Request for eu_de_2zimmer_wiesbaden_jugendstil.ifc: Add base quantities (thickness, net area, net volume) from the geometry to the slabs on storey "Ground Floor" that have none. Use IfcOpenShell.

First a look at what the model holds.

```python
import ifcopenshell
import ifcopenshell.util.element
import ifcopenshell.util.unit

model = ifcopenshell.open("eu_de_2zimmer_wiesbaden_jugendstil.ifc")
print(model.schema)
for unit_type in ("LENGTHUNIT", "AREAUNIT", "VOLUMEUNIT"):
    print(unit_type, ifcopenshell.util.unit.calculate_unit_scale(model, unit_type))
storey = next(s for s in model.by_type("IfcBuildingStorey") if s.Name == "Ground Floor")
slabs = [e for e in ifcopenshell.util.element.get_decomposition(storey) if e.is_a("IfcSlab")]
for e in sorted(slabs, key=lambda e: e.id()):
    print(e.id(), e.is_a(), e.Name, list(ifcopenshell.util.element.get_psets(e, qtos_only=True)), sep=" | ")
```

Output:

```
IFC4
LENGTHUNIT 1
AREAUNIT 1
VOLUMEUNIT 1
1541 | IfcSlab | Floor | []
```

```python
import ifcopenshell
import ifcopenshell.api.pset
import ifcopenshell.geom
import ifcopenshell.util.element
import ifcopenshell.util.shape
import ifcopenshell.util.unit

model = ifcopenshell.open("eu_de_2zimmer_wiesbaden_jugendstil.ifc")
unit_scale = ifcopenshell.util.unit.calculate_unit_scale(model)
area_scale = ifcopenshell.util.unit.calculate_unit_scale(model, "AREAUNIT")
volume_scale = ifcopenshell.util.unit.calculate_unit_scale(model, "VOLUMEUNIT")
settings = ifcopenshell.geom.settings()

storey = next(s for s in model.by_type("IfcBuildingStorey") if s.Name == "Ground Floor")
slabs = [e for e in ifcopenshell.util.element.get_decomposition(storey) if e.is_a("IfcSlab")]

for e in sorted(slabs, key=lambda e: e.id()):
    if ifcopenshell.util.element.get_psets(e, qtos_only=True, should_inherit=False):
        continue
    # Geometry comes back in metres, in the element's own axes.
    shape = ifcopenshell.geom.create_shape(settings, e)
    values = {
        "Width": ifcopenshell.util.shape.get_z(shape.geometry) / unit_scale,
        "NetArea": ifcopenshell.util.shape.get_footprint_area(shape.geometry) / area_scale,
        "NetVolume": ifcopenshell.util.shape.get_volume(shape.geometry) / volume_scale,
    }
    qto = ifcopenshell.api.pset.add_qto(model, product=e, name="Qto_SlabBaseQuantities")
    ifcopenshell.api.pset.edit_qto(model, qto=qto, properties=values)
    print(e.id(), {k: round(v, 3) for k, v in values.items()})

model.write("eu_de_2zimmer_wiesbaden_jugendstil_rev.ifc")
```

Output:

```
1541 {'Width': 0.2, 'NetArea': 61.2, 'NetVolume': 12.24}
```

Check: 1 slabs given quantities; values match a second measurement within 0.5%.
